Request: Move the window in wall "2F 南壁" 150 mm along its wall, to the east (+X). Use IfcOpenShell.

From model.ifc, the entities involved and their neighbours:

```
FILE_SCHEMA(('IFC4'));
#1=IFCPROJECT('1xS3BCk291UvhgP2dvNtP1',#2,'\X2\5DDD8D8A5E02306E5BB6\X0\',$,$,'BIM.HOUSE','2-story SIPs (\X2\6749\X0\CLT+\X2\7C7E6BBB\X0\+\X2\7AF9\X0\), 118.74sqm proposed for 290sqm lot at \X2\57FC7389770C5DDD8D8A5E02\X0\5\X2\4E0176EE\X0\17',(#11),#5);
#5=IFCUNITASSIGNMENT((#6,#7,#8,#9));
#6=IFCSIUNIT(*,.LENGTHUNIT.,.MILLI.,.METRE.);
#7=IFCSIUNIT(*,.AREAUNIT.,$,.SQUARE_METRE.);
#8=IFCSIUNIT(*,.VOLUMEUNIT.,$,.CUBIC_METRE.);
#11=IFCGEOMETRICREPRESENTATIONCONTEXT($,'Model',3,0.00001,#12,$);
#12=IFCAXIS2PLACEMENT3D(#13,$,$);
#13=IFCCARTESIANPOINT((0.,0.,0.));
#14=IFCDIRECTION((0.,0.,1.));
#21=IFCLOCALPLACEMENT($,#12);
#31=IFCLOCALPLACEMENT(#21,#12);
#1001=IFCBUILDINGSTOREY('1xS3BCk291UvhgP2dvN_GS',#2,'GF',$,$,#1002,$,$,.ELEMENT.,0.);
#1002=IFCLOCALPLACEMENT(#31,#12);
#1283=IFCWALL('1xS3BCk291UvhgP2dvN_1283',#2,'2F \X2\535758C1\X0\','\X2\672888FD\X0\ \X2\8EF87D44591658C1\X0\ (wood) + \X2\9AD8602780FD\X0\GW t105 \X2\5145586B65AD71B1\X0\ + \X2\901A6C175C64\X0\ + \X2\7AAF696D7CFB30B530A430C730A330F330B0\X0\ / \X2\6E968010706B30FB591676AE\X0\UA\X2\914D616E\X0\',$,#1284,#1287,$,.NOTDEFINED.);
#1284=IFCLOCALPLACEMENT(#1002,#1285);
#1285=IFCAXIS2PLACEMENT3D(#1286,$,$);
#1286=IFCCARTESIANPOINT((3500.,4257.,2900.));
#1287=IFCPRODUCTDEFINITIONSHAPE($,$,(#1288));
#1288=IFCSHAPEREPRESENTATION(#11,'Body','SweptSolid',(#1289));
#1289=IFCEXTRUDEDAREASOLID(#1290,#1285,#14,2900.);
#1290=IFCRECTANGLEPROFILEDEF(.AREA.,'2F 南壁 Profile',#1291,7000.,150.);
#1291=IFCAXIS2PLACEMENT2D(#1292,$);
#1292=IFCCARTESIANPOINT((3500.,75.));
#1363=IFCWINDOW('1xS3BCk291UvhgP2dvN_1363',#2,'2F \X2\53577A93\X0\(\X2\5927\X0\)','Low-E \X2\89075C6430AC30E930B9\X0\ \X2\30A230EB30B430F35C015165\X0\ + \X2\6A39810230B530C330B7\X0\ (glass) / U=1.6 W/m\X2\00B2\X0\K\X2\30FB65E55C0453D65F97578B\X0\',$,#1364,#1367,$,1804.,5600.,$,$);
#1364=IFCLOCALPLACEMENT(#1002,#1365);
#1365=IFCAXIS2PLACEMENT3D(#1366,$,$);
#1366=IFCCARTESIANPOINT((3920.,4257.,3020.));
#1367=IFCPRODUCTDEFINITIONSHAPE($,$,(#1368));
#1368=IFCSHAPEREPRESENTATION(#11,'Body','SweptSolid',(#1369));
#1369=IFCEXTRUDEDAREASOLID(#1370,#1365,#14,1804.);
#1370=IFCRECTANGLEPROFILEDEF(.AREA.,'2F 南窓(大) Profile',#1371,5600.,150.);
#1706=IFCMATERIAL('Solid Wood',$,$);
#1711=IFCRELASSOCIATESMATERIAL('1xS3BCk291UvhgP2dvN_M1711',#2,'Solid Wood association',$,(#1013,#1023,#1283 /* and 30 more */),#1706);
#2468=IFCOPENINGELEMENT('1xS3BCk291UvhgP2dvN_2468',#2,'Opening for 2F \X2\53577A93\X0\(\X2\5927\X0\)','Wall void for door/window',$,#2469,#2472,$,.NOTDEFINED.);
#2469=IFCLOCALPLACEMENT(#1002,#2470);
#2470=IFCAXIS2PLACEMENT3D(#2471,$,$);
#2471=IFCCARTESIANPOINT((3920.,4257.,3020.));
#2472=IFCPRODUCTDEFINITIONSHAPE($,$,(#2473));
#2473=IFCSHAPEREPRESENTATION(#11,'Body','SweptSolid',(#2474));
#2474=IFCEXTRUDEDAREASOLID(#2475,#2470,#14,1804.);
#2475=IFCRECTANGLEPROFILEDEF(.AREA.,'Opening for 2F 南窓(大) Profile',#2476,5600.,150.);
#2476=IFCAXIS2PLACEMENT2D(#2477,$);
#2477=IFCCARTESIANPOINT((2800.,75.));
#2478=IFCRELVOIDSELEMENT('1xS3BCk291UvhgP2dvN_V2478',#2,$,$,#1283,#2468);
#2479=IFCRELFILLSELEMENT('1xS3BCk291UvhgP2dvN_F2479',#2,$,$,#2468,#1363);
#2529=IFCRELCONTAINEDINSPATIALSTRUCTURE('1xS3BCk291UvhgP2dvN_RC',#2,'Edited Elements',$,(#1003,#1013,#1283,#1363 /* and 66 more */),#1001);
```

```python
import ifcopenshell
import ifcopenshell.api.geometry
import ifcopenshell.util.placement
import ifcopenshell.util.unit

model = ifcopenshell.open("model.ifc")
unit_scale = ifcopenshell.util.unit.calculate_unit_scale(model)

window = model.by_guid("1xS3BCk291UvhgP2dvN_1363")
opening = window.FillsVoids[0].RelatingOpeningElement
wall = opening.VoidsElements[0].RelatingBuildingElement

wall_matrix = ifcopenshell.util.placement.get_local_placement(wall.ObjectPlacement)
shift = wall_matrix[:3, 0] * 0.15 / unit_scale
before = ifcopenshell.util.placement.get_local_placement(window.ObjectPlacement)[:3, 3].copy()

# The window is not placed relative to its opening, so move both.
for product in (opening, window):
    matrix = ifcopenshell.util.placement.get_local_placement(product.ObjectPlacement)
    matrix[:3, 3] += shift
    ifcopenshell.api.geometry.edit_object_placement(model, product=product, matrix=matrix, is_si=False)

after = ifcopenshell.util.placement.get_local_placement(window.ObjectPlacement)[:3, 3]
print("window moved by", (after - before).round(3) + 0.0)

model.write("model_updated.ifc")
```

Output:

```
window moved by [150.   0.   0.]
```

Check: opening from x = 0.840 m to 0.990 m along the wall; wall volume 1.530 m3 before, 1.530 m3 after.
